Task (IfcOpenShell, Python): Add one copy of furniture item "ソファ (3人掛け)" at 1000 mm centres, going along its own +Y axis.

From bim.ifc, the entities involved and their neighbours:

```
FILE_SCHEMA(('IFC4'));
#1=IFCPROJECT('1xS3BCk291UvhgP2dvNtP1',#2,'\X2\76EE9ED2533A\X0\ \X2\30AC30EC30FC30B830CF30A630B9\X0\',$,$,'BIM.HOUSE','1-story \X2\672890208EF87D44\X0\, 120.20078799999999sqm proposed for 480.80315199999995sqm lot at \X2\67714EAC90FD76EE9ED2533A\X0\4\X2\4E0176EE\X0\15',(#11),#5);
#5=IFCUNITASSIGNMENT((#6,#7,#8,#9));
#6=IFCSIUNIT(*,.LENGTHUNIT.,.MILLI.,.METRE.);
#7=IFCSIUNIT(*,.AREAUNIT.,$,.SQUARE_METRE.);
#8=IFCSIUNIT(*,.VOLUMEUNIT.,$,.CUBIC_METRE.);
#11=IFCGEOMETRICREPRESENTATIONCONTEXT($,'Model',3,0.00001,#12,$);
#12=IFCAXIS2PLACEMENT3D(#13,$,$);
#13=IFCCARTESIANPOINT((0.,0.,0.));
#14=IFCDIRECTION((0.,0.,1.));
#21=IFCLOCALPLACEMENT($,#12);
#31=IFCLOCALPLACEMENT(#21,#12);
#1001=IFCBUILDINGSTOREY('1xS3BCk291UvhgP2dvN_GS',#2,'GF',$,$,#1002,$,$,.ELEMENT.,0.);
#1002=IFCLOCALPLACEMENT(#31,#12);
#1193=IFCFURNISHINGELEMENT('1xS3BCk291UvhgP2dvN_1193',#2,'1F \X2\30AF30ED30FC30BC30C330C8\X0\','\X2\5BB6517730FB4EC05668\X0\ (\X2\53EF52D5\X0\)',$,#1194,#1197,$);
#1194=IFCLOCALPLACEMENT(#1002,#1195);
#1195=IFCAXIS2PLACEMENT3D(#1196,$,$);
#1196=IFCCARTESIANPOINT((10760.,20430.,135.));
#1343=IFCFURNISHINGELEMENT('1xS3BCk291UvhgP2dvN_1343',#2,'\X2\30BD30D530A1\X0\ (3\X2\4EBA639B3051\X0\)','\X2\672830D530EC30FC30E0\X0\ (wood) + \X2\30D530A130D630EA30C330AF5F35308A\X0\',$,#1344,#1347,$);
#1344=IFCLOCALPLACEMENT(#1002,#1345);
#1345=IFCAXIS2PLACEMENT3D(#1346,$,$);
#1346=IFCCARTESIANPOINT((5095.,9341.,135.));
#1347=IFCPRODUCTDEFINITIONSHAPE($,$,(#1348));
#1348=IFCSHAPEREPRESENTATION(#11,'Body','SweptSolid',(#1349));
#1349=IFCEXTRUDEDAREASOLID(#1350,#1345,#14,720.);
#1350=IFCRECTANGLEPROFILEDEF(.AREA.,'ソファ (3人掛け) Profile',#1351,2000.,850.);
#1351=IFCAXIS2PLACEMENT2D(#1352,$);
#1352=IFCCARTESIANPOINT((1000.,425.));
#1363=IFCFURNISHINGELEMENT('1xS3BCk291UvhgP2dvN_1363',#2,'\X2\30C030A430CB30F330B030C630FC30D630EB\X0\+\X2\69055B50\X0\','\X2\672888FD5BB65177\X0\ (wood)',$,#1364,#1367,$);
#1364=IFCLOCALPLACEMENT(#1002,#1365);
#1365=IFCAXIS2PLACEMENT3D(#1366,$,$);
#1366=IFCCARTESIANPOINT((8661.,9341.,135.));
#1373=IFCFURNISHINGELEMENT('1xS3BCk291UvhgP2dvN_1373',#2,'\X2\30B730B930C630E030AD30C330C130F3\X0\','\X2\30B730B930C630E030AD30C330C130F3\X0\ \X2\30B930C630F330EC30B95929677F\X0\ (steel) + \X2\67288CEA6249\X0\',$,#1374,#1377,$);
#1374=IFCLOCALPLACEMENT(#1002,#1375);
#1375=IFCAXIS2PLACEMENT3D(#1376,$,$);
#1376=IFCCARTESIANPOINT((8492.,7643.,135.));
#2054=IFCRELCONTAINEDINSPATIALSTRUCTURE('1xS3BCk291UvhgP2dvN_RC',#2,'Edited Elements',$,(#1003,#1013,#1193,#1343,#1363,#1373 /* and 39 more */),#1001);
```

```python
import ifcopenshell
import ifcopenshell.api.geometry
import ifcopenshell.api.root
import ifcopenshell.util.element
import ifcopenshell.util.placement
import ifcopenshell.util.unit

model = ifcopenshell.open("bim.ifc")
unit_scale = ifcopenshell.util.unit.calculate_unit_scale(model)


def reuse_history(source, copy):
    """copy_class also copies each property set's owner history, people and application; keep the originals."""
    for rel in copy.IsDefinedBy:
        if rel.is_a("IfcRelDefinesByProperties") and (history := rel.RelatingPropertyDefinition.OwnerHistory):
            rel.RelatingPropertyDefinition.OwnerHistory = source.OwnerHistory
            ifcopenshell.util.element.remove_deep2(model, history)


source = model.by_id(1343)
base = ifcopenshell.util.placement.get_local_placement(source.ObjectPlacement)
step = base[:3, 1] * 1 / unit_scale

for i in range(1, 2):
    copy = ifcopenshell.api.root.copy_class(model, product=source)
    copy.Representation = ifcopenshell.util.element.copy_deep(
        model, source.Representation, exclude=["IfcGeometricRepresentationContext", "IfcRepresentationMap"]
    )
    reuse_history(source, copy)
    matrix = base.copy()
    matrix[:3, 3] += i * step
    print("added at", matrix[:3, 3].round(3) + 0.0)
    ifcopenshell.api.geometry.edit_object_placement(model, product=copy, matrix=matrix, is_si=False)

model.write("bim_edited.ifc")
```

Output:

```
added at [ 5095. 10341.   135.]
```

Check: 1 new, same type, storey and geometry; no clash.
